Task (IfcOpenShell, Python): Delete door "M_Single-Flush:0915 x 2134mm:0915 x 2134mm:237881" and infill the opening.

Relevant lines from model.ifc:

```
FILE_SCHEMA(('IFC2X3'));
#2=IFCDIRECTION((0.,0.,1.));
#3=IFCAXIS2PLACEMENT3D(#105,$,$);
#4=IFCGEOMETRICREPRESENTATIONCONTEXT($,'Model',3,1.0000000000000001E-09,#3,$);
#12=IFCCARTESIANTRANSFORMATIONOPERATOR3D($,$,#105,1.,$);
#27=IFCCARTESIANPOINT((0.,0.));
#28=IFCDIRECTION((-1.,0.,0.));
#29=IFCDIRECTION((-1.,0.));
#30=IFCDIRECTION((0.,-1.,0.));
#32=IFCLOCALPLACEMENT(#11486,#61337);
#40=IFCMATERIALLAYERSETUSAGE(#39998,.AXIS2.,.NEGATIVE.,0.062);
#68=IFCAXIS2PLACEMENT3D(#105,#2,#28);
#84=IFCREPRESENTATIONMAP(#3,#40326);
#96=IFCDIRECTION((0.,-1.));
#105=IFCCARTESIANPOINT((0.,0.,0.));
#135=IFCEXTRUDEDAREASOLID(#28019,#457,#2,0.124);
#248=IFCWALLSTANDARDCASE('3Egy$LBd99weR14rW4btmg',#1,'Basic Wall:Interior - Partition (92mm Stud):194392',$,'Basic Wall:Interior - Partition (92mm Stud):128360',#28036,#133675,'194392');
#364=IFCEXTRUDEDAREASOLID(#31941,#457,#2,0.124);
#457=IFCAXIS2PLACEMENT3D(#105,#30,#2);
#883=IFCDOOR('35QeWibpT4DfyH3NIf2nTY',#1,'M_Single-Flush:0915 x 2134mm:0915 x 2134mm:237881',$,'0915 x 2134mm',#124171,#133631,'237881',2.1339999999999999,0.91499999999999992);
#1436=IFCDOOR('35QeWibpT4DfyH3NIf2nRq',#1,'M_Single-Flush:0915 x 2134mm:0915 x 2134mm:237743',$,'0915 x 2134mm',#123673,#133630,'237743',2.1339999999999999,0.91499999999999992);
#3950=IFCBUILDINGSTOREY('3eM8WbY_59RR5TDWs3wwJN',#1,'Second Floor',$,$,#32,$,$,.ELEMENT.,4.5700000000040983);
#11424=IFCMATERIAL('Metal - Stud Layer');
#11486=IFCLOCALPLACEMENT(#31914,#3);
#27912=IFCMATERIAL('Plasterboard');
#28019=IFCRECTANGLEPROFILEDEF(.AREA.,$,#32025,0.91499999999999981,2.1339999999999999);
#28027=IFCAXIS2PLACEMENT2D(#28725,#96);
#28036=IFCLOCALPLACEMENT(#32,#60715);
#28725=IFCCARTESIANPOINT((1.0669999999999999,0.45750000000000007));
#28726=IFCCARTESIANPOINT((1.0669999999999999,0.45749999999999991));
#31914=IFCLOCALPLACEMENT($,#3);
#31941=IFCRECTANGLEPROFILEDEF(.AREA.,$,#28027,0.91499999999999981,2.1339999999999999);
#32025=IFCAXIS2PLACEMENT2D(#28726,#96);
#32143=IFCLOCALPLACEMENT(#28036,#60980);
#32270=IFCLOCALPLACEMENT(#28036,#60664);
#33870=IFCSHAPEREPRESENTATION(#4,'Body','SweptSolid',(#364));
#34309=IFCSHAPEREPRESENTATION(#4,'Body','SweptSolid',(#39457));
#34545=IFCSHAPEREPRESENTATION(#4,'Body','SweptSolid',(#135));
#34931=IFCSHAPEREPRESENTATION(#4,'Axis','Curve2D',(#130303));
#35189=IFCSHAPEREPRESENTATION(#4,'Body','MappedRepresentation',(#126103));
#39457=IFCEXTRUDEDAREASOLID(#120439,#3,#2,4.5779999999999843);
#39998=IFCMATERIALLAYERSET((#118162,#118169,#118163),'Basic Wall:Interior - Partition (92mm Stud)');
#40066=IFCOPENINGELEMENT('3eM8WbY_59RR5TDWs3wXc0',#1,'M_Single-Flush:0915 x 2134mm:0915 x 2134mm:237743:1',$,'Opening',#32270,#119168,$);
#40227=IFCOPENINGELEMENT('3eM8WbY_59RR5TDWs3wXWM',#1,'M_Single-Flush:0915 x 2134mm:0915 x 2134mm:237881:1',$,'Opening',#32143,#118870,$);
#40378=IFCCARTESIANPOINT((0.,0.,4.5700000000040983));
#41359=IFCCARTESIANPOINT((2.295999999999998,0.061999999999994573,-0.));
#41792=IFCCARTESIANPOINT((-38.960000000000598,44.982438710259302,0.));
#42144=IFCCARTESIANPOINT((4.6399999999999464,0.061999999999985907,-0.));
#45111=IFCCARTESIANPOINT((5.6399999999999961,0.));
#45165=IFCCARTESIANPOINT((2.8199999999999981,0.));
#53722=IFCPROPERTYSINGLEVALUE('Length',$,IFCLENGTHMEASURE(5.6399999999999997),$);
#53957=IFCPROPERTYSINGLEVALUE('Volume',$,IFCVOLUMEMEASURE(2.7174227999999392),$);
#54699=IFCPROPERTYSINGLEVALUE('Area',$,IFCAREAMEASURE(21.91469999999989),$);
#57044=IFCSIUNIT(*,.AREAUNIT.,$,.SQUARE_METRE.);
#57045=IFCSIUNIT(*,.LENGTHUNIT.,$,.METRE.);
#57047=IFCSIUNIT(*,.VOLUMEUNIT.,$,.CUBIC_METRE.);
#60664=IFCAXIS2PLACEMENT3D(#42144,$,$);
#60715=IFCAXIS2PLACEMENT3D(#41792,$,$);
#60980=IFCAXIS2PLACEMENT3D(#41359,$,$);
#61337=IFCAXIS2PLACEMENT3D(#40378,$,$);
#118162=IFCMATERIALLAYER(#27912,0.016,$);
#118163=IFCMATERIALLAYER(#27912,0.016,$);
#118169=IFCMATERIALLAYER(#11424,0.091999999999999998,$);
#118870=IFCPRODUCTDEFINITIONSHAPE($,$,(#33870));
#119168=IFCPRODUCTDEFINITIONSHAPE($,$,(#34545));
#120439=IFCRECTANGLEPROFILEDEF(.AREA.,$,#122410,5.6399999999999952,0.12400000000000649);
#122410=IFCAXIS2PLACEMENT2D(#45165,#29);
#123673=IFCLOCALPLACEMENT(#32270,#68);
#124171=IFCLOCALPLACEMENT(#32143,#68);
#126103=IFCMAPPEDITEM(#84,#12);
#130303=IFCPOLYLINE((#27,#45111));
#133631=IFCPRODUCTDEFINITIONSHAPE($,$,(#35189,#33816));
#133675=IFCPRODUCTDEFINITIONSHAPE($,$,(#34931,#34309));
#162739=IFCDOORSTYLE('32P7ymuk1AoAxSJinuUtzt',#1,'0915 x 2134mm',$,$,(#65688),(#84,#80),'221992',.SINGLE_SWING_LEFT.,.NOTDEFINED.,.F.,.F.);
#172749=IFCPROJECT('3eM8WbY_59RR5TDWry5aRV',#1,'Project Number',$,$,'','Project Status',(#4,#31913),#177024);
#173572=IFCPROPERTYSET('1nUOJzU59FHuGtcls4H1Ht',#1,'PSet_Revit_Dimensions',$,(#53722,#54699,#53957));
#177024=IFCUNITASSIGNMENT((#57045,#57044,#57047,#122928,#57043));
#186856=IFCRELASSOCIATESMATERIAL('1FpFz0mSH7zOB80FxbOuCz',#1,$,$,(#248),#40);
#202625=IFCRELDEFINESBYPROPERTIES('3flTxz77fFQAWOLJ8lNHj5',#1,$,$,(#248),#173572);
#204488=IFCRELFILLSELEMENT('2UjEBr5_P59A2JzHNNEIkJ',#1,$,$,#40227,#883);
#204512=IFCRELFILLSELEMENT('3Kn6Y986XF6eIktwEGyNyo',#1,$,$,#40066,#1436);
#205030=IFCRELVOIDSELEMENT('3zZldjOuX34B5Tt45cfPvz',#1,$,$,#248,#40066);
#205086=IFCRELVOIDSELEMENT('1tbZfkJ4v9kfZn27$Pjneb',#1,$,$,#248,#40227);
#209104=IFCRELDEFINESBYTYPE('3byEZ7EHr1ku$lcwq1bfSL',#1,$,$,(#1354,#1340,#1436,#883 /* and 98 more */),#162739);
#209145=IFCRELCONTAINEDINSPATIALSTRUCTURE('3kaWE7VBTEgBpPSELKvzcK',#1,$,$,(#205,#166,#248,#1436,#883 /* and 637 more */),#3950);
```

```python
import ifcopenshell
import ifcopenshell.api.feature
import ifcopenshell.api.pset
import ifcopenshell.api.root
import ifcopenshell.geom
import ifcopenshell.util.element
import ifcopenshell.util.shape
import ifcopenshell.util.unit

model = ifcopenshell.open("model.ifc")
area_scale = ifcopenshell.util.unit.calculate_unit_scale(model, "AREAUNIT")
volume_scale = ifcopenshell.util.unit.calculate_unit_scale(model, "VOLUMEUNIT")
settings = ifcopenshell.geom.settings()


def volume(element):
    """Net volume in cubic metres, openings subtracted."""
    shape = ifcopenshell.geom.create_shape(settings, element)
    return ifcopenshell.util.shape.get_volume(shape.geometry)


door = model.by_guid("35QeWibpT4DfyH3NIf2nTY")
opening = door.FillsVoids[0].RelatingOpeningElement
wall = opening.VoidsElements[0].RelatingBuildingElement
before = volume(wall)

ifcopenshell.api.root.remove_product(model, product=door)
ifcopenshell.api.feature.remove_feature(model, feature=opening)

after = volume(wall)
thickness = 0.124  # wall thickness in metres

# Update the wall's stored quantities.
pset = model.by_id(ifcopenshell.util.element.get_pset(wall, "PSet_Revit_Dimensions", should_inherit=False)["id"])
ifcopenshell.api.pset.edit_pset(model, pset=pset, properties={
    "Area": model.create_entity("IfcAreaMeasure", after / thickness / area_scale),
    "Volume": model.create_entity("IfcVolumeMeasure", after / volume_scale),
})

print(f"wall volume {before:.3f} -> {after:.3f} m3")

model.write("model_updated.ifc")
```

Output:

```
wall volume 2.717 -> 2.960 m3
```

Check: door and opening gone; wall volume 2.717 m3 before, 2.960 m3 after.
